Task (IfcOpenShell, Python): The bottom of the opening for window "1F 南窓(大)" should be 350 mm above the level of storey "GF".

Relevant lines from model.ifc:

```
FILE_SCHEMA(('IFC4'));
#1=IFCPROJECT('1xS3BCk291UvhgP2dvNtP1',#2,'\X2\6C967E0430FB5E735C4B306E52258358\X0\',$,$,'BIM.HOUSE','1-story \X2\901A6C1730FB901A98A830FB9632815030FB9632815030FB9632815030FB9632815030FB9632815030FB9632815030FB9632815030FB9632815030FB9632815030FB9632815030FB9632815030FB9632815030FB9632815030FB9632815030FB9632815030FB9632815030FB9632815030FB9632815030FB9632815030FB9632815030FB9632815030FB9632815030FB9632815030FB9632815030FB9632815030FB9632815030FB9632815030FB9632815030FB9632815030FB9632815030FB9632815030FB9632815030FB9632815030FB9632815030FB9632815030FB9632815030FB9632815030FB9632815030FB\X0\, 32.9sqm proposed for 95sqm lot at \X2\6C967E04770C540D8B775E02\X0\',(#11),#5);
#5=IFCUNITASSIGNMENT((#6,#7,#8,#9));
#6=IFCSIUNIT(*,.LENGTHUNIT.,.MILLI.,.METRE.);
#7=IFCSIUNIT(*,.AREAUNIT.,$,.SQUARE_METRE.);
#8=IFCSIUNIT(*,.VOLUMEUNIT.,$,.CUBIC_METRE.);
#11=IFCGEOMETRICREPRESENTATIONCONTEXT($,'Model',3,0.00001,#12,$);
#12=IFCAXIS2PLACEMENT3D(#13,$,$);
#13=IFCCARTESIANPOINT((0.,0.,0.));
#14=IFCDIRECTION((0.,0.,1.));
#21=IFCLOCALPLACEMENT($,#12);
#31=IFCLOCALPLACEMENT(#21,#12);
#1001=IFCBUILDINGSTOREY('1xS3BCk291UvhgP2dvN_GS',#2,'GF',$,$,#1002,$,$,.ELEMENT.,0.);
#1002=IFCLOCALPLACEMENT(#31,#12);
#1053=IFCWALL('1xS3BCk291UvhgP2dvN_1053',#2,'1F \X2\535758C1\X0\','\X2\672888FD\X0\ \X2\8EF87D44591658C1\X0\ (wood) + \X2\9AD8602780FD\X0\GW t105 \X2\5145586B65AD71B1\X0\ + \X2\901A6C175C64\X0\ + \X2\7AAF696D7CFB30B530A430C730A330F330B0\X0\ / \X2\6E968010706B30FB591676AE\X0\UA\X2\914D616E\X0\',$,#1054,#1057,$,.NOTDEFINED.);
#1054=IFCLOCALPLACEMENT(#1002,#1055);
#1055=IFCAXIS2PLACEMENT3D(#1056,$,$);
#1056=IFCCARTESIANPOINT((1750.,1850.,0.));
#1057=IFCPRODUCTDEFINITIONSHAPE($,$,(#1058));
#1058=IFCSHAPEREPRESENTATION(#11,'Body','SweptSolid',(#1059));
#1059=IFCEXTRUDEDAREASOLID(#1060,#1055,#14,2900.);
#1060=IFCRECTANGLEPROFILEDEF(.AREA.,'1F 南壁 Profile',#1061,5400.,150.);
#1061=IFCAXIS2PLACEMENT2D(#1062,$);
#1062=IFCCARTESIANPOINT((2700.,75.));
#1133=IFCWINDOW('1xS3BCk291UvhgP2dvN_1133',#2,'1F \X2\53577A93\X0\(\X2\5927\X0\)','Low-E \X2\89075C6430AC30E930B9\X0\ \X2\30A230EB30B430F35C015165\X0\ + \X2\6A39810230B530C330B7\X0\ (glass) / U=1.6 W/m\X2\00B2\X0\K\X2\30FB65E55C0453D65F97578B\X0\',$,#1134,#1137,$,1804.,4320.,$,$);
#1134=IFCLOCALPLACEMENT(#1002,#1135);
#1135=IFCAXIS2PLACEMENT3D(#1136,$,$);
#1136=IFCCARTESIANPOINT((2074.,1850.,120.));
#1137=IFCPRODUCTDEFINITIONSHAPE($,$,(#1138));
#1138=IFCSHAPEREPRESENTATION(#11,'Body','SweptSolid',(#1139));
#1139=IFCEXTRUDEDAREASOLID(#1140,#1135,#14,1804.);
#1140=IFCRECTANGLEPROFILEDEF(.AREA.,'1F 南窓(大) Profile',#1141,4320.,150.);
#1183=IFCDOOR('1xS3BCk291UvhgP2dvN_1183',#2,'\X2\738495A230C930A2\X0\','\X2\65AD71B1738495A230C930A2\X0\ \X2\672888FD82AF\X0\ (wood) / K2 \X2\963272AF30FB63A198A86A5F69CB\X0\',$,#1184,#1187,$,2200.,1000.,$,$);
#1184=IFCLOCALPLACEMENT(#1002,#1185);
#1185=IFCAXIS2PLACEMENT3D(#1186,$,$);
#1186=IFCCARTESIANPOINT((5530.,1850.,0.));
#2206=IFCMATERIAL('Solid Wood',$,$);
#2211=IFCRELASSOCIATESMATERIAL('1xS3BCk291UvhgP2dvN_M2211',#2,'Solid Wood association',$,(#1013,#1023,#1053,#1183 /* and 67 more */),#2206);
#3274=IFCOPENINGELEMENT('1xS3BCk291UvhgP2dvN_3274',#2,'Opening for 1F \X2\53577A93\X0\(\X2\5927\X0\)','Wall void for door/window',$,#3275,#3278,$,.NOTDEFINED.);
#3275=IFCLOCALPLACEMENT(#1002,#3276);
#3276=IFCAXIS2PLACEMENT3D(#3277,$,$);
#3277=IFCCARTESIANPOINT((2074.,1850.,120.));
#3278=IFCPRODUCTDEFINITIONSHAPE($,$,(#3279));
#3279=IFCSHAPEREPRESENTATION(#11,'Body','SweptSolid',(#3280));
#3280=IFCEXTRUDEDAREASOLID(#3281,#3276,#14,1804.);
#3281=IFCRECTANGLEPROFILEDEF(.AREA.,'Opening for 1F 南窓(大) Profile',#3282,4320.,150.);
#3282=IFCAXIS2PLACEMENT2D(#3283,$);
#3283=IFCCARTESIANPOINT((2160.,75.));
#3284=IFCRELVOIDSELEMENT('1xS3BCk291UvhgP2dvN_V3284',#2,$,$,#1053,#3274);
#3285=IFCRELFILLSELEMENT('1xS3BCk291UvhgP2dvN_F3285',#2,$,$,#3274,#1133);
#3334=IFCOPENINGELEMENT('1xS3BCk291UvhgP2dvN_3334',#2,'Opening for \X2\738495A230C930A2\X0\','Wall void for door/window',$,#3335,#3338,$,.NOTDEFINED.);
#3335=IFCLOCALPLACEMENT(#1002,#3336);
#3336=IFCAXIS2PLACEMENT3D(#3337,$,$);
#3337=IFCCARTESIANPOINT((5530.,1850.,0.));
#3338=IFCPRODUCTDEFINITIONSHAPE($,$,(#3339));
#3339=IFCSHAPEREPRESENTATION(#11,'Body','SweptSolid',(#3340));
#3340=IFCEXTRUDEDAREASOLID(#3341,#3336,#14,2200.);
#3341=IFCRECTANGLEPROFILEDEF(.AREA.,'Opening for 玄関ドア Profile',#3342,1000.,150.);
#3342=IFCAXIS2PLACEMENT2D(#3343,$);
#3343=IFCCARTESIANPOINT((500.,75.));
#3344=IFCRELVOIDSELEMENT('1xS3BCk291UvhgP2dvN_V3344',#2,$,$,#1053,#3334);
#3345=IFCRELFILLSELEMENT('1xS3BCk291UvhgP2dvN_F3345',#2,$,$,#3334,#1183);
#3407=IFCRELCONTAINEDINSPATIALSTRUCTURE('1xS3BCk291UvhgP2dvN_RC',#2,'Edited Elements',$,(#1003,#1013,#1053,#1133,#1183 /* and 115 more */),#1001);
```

```python
import numpy as np
import ifcopenshell
import ifcopenshell.api.geometry
import ifcopenshell.geom
import ifcopenshell.util.element
import ifcopenshell.util.placement
import ifcopenshell.util.shape
import ifcopenshell.util.unit

model = ifcopenshell.open("model.ifc")
unit_scale = ifcopenshell.util.unit.calculate_unit_scale(model)

window = model.by_guid("1xS3BCk291UvhgP2dvN_1133")
opening = window.FillsVoids[0].RelatingOpeningElement
storey = ifcopenshell.util.element.get_container(window, ifc_class="IfcBuildingStorey")
level = ifcopenshell.util.placement.get_local_placement(storey.ObjectPlacement)[2, 3]

# The opening's origin need not be at the sill, so measure its lowest point.
shape = ifcopenshell.geom.create_shape(ifcopenshell.geom.settings(), opening)
bottom = ifcopenshell.util.shape.get_shape_bottom_elevation(shape, shape.geometry) / unit_scale
dz = level + 350.0 - bottom

shift = np.array([0.0, 0.0, dz])
# The window is not placed relative to its opening, so move both.
for product in (opening, window):
    matrix = ifcopenshell.util.placement.get_local_placement(product.ObjectPlacement)
    matrix[:3, 3] += shift
    ifcopenshell.api.geometry.edit_object_placement(model, product=product, matrix=matrix, is_si=False)

print(f"moved by {dz * unit_scale:+.3f} m")

model.write("model_v2.ifc")
```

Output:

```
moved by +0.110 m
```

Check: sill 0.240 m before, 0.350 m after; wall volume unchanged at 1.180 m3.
